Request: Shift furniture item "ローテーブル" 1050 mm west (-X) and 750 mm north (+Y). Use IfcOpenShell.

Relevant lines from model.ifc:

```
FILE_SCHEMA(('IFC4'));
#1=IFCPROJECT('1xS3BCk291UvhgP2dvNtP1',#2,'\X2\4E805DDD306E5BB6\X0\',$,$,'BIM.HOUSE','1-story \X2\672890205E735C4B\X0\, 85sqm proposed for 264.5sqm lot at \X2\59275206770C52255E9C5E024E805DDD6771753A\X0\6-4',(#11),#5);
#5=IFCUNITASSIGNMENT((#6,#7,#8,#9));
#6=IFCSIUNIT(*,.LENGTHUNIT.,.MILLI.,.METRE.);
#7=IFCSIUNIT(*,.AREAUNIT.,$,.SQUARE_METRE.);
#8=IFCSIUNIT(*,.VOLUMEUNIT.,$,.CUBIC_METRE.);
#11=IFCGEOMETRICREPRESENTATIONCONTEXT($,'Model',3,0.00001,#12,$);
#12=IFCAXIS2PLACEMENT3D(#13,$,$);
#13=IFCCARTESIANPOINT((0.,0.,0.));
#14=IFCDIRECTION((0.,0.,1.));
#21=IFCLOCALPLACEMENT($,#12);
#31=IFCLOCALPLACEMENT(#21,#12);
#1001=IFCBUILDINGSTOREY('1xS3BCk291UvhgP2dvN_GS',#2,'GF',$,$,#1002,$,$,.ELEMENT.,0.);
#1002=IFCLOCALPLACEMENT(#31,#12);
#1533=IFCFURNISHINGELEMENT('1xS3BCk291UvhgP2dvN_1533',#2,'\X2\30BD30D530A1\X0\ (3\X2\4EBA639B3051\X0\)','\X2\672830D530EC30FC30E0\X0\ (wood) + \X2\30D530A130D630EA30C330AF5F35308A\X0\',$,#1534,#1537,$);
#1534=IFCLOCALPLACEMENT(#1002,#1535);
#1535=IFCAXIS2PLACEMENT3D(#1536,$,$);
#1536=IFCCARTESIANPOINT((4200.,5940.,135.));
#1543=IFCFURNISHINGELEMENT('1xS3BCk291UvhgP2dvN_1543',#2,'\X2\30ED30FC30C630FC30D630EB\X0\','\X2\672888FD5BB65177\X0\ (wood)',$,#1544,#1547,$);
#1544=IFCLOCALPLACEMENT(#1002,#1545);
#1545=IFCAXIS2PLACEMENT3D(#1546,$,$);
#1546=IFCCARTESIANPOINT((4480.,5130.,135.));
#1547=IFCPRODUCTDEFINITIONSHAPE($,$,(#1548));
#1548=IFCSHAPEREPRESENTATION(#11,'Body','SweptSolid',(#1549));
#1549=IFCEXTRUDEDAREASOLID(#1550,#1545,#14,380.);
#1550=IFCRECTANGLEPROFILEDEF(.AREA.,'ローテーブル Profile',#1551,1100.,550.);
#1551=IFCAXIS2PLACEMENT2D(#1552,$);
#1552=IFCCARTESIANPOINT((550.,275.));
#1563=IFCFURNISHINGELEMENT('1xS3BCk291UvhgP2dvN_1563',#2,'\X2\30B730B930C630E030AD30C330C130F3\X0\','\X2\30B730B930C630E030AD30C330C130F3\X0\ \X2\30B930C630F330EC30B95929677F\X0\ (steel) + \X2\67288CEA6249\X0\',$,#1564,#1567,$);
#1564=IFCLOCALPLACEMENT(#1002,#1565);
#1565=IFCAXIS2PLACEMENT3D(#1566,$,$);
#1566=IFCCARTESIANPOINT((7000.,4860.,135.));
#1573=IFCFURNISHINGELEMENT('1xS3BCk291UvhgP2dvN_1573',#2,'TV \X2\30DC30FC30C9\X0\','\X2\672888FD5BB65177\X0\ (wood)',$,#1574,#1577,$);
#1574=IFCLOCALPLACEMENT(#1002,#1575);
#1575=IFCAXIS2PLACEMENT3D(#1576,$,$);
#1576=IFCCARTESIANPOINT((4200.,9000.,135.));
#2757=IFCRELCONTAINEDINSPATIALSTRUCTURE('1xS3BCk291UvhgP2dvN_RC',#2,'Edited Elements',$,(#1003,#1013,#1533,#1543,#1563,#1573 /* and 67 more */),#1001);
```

```python
import ifcopenshell
import ifcopenshell.api.geometry
import ifcopenshell.util.placement
import ifcopenshell.util.unit

model = ifcopenshell.open("model.ifc")
unit_scale = ifcopenshell.util.unit.calculate_unit_scale(model)

item = model.by_guid("1xS3BCk291UvhgP2dvN_1543")
matrix = ifcopenshell.util.placement.get_local_placement(item.ObjectPlacement)
matrix[0, 3] -= 1.05 / unit_scale
matrix[1, 3] += 0.75 / unit_scale
ifcopenshell.api.geometry.edit_object_placement(model, product=item, matrix=matrix, is_si=False)

print(ifcopenshell.util.placement.get_local_placement(item.ObjectPlacement).round(3) + 0.0)

model.write("model_rev.ifc")
```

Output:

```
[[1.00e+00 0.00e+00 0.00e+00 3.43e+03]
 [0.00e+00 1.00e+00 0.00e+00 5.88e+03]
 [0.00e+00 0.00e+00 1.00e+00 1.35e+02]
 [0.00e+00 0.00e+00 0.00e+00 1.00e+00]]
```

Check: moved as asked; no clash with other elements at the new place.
